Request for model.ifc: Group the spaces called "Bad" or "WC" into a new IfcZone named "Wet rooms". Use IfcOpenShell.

First a look at what the model holds.

```python
import ifcopenshell

model = ifcopenshell.open("model.ifc")
print(model.schema)
seen = {}
for space in model.by_type("IfcSpace"):
    seen[space.LongName] = seen.get(space.LongName, 0) + 1
for name, count in sorted(seen.items(), key=str):
    print(count, "x", name)
print("zones:", [z.Name for z in model.by_type("IfcZone")][:20])
```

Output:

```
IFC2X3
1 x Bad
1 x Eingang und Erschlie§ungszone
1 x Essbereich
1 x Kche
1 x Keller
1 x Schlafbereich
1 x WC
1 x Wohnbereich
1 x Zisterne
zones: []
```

```python
import ifcopenshell
import ifcopenshell.api.group
import ifcopenshell.api.root

model = ifcopenshell.open("model.ifc")

names = {"Bad", "WC"}
spaces = [s for s in model.by_type("IfcSpace") if s.LongName in names]

zone = ifcopenshell.api.root.create_entity(model, ifc_class="IfcZone", name="Wet rooms")
ifcopenshell.api.group.assign_group(model, products=spaces, group=zone)
print(len(spaces), "spaces in", zone.Name)

model.write("model-out.ifc")
```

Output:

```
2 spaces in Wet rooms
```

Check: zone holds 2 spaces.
